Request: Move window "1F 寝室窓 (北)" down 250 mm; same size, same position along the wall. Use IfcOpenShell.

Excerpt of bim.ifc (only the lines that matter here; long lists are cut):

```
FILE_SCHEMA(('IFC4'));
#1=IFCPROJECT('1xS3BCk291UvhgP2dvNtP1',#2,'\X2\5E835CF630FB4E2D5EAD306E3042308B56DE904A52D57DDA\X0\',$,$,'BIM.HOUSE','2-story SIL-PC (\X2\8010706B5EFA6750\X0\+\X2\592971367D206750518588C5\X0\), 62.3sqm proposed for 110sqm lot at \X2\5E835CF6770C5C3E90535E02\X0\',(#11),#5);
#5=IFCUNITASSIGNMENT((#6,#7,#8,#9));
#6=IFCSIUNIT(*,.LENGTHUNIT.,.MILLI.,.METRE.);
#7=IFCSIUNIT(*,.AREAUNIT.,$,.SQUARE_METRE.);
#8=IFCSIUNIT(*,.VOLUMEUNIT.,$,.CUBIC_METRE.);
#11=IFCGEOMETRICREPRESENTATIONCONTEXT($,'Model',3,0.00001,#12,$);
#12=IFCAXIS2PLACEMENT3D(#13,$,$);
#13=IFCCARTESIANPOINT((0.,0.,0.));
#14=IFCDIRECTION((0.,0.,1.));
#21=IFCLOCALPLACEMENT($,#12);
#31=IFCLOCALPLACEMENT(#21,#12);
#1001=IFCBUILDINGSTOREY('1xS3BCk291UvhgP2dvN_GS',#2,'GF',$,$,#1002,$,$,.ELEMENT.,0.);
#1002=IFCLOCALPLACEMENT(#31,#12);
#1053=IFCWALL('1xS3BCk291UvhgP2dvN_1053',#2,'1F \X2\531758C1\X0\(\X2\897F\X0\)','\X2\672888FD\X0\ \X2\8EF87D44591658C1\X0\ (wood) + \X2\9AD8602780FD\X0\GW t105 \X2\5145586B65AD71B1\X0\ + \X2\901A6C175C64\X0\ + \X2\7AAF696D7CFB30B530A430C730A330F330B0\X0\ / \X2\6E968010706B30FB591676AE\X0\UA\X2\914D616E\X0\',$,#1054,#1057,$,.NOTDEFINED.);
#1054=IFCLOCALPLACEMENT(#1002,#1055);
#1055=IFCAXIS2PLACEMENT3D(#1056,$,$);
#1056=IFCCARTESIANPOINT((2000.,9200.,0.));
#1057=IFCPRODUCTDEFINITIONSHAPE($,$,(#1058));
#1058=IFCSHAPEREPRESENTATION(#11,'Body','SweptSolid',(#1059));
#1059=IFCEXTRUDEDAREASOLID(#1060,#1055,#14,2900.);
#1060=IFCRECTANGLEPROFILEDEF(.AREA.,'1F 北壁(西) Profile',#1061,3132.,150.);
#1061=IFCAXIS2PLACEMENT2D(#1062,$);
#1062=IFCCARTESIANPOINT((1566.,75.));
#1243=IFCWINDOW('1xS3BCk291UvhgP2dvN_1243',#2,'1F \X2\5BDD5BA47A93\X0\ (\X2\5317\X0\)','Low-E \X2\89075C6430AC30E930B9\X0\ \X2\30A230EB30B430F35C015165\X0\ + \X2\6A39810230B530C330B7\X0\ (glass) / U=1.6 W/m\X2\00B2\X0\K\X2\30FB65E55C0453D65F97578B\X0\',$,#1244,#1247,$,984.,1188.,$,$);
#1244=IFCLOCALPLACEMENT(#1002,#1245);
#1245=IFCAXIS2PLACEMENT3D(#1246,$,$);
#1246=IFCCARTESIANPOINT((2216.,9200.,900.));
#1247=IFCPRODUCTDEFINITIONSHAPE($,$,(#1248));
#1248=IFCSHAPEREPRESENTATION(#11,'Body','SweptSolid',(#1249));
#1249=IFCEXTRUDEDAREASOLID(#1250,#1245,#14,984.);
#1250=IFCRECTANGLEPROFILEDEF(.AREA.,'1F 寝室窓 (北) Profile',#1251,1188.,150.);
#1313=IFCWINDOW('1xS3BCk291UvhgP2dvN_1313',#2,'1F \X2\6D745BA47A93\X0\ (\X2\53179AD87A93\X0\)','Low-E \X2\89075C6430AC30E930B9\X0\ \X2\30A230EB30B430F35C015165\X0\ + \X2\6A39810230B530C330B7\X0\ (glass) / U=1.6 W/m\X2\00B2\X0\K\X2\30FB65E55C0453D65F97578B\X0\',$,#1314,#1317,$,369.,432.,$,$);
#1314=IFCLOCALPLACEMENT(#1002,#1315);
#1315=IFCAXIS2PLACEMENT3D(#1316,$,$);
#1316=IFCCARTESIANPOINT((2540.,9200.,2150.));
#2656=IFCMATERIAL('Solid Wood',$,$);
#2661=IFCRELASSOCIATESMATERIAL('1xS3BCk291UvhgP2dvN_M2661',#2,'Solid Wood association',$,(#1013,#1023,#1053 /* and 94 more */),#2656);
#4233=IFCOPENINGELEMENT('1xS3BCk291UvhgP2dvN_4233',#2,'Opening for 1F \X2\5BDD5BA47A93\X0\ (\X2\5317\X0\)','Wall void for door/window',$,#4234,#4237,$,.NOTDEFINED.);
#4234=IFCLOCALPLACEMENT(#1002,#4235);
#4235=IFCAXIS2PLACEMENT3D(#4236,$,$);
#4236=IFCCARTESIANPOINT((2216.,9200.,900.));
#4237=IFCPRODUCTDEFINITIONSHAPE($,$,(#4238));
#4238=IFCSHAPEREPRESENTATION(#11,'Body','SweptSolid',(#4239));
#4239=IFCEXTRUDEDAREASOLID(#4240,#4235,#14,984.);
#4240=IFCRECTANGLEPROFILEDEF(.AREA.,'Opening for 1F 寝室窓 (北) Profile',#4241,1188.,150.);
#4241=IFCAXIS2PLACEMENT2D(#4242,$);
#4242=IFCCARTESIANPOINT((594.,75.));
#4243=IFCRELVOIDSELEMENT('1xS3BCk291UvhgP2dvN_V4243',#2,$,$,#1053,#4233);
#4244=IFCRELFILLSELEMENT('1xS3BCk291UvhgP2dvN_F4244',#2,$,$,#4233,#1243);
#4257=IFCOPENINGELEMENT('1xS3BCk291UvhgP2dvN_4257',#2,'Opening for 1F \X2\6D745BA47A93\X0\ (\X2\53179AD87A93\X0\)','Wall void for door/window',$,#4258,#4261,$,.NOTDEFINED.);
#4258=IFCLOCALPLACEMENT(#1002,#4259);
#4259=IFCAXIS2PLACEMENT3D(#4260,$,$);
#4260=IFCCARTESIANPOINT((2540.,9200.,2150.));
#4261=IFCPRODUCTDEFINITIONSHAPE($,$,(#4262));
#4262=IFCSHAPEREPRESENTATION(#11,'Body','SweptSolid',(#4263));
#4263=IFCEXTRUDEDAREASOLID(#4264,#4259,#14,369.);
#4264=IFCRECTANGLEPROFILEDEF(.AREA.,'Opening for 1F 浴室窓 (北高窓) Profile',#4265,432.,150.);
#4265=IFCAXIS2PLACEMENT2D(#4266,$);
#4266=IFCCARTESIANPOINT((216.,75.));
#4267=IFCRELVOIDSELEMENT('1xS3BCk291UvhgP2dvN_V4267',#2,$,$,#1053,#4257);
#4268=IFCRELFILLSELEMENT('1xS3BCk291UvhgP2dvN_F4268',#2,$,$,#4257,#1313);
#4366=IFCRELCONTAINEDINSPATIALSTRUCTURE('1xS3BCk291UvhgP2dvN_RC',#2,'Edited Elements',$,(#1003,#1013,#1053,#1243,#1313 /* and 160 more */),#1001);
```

```python
import numpy as np
import ifcopenshell
import ifcopenshell.api.geometry
import ifcopenshell.util.placement
import ifcopenshell.util.unit

model = ifcopenshell.open("bim.ifc")
unit_scale = ifcopenshell.util.unit.calculate_unit_scale(model)

window = model.by_guid("1xS3BCk291UvhgP2dvN_1243")
opening = window.FillsVoids[0].RelatingOpeningElement
dz = -250.0

shift = np.array([0.0, 0.0, dz])
# The window is not placed relative to its opening, so move both.
for product in (opening, window):
    matrix = ifcopenshell.util.placement.get_local_placement(product.ObjectPlacement)
    matrix[:3, 3] += shift
    ifcopenshell.api.geometry.edit_object_placement(model, product=product, matrix=matrix, is_si=False)

print(f"moved by {dz * unit_scale:+.3f} m")

model.write("bim_v2.ifc")
```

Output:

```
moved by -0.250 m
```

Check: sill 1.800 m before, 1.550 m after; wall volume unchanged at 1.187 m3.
